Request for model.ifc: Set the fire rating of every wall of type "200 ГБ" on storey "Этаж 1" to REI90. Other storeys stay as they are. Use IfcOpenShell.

First a look at what the model holds.

```python
import ifcopenshell
import ifcopenshell.util.element

model = ifcopenshell.open("model.ifc")
print(model.schema)
storey = next(s for s in model.by_type("IfcBuildingStorey") if s.Name == "Этаж 1")
walls = [e for e in ifcopenshell.util.element.get_decomposition(storey) if e.is_a("IfcWall")]
seen = {}
for e in walls:
    element_type = ifcopenshell.util.element.get_type(e)
    key = (element_type.Name if element_type != e and element_type else None, ifcopenshell.util.element.get_pset(e, "Pset_WallCommon", "FireRating"))
    seen[key] = seen.get(key, 0) + 1
for (name, value), count in sorted(seen.items(), key=str):
    print(count, "x", name, "|", value)
```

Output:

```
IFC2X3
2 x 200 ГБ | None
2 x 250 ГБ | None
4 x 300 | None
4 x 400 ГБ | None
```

```python
import ifcopenshell
import ifcopenshell.api.pset
import ifcopenshell.util.element

model = ifcopenshell.open("model.ifc")

storey = next(s for s in model.by_type("IfcBuildingStorey") if s.Name == "Этаж 1")
walls = [e for e in ifcopenshell.util.element.get_decomposition(storey) if e.is_a("IfcWall")]

count = 0
for e in walls:
    element_type = ifcopenshell.util.element.get_type(e)
    if element_type in (None, e) or element_type.Name != "200 ГБ":
        continue
    # add_pset returns the element's existing set when there is one.
    pset = ifcopenshell.api.pset.add_pset(model, product=e, name="Pset_WallCommon")
    ifcopenshell.api.pset.edit_pset(model, pset=pset, properties={"FireRating": "REI90"})
    count += 1

print(count, "walls updated")

model.write("model_rev.ifc")
```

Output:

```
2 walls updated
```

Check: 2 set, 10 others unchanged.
